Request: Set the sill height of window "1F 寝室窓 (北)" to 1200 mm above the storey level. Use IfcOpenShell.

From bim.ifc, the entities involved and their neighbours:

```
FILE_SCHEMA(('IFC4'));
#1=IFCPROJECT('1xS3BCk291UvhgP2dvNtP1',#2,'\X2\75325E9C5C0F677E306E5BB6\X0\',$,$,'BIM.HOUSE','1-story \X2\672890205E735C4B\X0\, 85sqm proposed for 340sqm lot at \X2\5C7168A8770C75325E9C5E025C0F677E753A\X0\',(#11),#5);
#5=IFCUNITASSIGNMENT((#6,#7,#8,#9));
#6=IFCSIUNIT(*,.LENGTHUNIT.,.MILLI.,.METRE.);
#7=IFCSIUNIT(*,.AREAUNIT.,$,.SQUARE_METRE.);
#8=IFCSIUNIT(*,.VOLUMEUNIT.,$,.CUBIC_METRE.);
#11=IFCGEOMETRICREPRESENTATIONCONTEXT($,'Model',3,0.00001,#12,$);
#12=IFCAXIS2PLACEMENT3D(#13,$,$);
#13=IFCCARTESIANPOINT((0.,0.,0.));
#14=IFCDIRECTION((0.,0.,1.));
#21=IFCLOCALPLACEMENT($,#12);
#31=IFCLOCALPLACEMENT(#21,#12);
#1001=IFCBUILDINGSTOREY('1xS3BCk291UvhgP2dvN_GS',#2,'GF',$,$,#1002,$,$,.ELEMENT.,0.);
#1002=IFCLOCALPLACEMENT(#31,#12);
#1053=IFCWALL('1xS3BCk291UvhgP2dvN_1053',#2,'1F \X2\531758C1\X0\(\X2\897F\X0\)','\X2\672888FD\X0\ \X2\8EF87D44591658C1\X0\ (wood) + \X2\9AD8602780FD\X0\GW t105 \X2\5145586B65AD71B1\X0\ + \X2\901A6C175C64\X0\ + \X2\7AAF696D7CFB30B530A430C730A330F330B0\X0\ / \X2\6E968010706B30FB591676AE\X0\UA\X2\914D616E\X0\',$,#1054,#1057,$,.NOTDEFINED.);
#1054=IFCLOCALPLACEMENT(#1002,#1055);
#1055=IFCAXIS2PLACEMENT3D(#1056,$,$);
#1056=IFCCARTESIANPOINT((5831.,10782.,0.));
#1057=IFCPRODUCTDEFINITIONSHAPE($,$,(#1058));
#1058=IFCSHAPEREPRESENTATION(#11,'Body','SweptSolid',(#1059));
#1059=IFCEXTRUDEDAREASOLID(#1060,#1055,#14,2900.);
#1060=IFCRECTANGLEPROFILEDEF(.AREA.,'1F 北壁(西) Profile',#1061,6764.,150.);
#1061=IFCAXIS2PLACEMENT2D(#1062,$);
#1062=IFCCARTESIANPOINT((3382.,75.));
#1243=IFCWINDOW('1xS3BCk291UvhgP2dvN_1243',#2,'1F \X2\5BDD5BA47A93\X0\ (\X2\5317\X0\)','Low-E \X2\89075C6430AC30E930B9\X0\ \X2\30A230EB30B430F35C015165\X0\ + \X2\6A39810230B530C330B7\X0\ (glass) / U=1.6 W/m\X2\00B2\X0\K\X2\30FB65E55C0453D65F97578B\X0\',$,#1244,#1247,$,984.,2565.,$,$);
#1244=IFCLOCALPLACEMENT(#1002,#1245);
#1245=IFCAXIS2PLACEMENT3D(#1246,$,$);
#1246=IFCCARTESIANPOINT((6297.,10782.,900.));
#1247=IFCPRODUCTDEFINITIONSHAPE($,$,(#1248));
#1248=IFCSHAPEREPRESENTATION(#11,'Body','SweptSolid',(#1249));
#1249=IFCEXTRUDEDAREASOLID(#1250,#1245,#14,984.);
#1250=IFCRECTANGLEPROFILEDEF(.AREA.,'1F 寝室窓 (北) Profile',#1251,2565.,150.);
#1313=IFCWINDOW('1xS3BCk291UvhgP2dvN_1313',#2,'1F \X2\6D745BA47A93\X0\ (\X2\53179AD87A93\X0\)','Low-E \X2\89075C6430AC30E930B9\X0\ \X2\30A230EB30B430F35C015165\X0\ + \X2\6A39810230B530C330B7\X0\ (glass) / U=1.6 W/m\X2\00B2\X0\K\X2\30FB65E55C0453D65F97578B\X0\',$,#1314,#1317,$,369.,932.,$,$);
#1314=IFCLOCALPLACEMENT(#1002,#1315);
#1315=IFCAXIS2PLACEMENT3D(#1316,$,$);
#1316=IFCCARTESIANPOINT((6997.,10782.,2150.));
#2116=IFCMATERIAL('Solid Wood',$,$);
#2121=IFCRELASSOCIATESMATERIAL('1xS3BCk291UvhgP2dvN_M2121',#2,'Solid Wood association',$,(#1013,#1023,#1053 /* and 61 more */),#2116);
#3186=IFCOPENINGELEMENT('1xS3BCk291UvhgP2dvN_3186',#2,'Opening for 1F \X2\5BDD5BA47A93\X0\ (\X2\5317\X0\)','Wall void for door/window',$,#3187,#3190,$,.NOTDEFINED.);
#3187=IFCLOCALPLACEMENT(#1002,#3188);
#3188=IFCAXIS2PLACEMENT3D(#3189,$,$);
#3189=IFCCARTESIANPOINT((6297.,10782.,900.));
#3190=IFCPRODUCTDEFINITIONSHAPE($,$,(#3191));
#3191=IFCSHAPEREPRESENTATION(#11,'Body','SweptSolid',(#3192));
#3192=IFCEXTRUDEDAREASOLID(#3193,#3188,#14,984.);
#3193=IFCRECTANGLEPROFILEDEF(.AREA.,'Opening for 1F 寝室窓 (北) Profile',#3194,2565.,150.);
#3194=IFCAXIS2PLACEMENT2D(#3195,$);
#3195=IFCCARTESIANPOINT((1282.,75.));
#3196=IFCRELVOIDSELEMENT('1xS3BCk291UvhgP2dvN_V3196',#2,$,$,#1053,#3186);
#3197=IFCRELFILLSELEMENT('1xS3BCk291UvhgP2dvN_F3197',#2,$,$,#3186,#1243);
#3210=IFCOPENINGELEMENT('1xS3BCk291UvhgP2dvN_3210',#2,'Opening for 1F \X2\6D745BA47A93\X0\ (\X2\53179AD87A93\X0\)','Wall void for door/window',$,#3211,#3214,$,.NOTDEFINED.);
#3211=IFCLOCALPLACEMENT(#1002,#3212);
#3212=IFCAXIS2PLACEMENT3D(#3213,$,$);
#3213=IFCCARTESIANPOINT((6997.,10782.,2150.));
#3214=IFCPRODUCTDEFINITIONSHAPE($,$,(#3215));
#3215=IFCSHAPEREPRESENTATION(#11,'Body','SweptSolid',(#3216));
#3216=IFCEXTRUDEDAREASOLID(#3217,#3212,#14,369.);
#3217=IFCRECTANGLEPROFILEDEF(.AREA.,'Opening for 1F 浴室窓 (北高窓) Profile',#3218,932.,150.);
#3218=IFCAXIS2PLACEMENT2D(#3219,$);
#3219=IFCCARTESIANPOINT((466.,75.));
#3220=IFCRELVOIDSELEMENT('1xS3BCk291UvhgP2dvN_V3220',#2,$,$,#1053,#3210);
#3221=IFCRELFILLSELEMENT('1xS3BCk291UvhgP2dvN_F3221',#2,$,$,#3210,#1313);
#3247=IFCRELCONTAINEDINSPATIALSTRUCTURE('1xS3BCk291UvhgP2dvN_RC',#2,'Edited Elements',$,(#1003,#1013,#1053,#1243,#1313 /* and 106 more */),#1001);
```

```python
import numpy as np
import ifcopenshell
import ifcopenshell.api.geometry
import ifcopenshell.geom
import ifcopenshell.util.element
import ifcopenshell.util.placement
import ifcopenshell.util.shape
import ifcopenshell.util.unit

model = ifcopenshell.open("bim.ifc")
unit_scale = ifcopenshell.util.unit.calculate_unit_scale(model)

window = model.by_guid("1xS3BCk291UvhgP2dvN_1243")
opening = window.FillsVoids[0].RelatingOpeningElement
storey = ifcopenshell.util.element.get_container(window, ifc_class="IfcBuildingStorey")
level = ifcopenshell.util.placement.get_local_placement(storey.ObjectPlacement)[2, 3]

# The opening's origin need not be at the sill, so measure its lowest point.
shape = ifcopenshell.geom.create_shape(ifcopenshell.geom.settings(), opening)
bottom = ifcopenshell.util.shape.get_shape_bottom_elevation(shape, shape.geometry) / unit_scale
dz = level + 1.2 / unit_scale - bottom

shift = np.array([0.0, 0.0, dz])
# The window is not placed relative to its opening, so move both.
for product in (opening, window):
    matrix = ifcopenshell.util.placement.get_local_placement(product.ObjectPlacement)
    matrix[:3, 3] += shift
    ifcopenshell.api.geometry.edit_object_placement(model, product=product, matrix=matrix, is_si=False)

print(f"moved by {dz * unit_scale:+.3f} m")

model.write("bim-out.ifc")
```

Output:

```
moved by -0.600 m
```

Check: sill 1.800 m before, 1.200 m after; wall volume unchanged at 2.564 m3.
